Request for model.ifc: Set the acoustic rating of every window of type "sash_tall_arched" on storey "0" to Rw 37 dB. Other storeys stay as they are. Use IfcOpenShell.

First a look at what the model holds.

```python
import ifcopenshell
import ifcopenshell.util.element

model = ifcopenshell.open("model.ifc")
print(model.schema)
storey = next(s for s in model.by_type("IfcBuildingStorey") if s.Name == "0")
windows = [e for e in ifcopenshell.util.element.get_decomposition(storey) if e.is_a("IfcWindow")]
seen = {}
for e in windows:
    element_type = ifcopenshell.util.element.get_type(e)
    key = (element_type.Name if element_type != e and element_type else None, ifcopenshell.util.element.get_pset(e, "Pset_WindowCommon", "AcousticRating"))
    seen[key] = seen.get(key, 0) + 1
for (name, value), count in sorted(seen.items(), key=str):
    print(count, "x", name, "|", value)
```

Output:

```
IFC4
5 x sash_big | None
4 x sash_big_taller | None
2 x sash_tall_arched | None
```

```python
import ifcopenshell
import ifcopenshell.api.pset
import ifcopenshell.util.element

model = ifcopenshell.open("model.ifc")

storey = next(s for s in model.by_type("IfcBuildingStorey") if s.Name == "0")
windows = [e for e in ifcopenshell.util.element.get_decomposition(storey) if e.is_a("IfcWindow")]

count = 0
for e in windows:
    element_type = ifcopenshell.util.element.get_type(e)
    if element_type in (None, e) or element_type.Name != "sash_tall_arched":
        continue
    # add_pset returns the element's existing set when there is one.
    pset = ifcopenshell.api.pset.add_pset(model, product=e, name="Pset_WindowCommon")
    ifcopenshell.api.pset.edit_pset(model, pset=pset, properties={"AcousticRating": "Rw 37 dB"})
    count += 1

print(count, "windows updated")

model.write("model_rev.ifc")
```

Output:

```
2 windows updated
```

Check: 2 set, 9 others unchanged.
